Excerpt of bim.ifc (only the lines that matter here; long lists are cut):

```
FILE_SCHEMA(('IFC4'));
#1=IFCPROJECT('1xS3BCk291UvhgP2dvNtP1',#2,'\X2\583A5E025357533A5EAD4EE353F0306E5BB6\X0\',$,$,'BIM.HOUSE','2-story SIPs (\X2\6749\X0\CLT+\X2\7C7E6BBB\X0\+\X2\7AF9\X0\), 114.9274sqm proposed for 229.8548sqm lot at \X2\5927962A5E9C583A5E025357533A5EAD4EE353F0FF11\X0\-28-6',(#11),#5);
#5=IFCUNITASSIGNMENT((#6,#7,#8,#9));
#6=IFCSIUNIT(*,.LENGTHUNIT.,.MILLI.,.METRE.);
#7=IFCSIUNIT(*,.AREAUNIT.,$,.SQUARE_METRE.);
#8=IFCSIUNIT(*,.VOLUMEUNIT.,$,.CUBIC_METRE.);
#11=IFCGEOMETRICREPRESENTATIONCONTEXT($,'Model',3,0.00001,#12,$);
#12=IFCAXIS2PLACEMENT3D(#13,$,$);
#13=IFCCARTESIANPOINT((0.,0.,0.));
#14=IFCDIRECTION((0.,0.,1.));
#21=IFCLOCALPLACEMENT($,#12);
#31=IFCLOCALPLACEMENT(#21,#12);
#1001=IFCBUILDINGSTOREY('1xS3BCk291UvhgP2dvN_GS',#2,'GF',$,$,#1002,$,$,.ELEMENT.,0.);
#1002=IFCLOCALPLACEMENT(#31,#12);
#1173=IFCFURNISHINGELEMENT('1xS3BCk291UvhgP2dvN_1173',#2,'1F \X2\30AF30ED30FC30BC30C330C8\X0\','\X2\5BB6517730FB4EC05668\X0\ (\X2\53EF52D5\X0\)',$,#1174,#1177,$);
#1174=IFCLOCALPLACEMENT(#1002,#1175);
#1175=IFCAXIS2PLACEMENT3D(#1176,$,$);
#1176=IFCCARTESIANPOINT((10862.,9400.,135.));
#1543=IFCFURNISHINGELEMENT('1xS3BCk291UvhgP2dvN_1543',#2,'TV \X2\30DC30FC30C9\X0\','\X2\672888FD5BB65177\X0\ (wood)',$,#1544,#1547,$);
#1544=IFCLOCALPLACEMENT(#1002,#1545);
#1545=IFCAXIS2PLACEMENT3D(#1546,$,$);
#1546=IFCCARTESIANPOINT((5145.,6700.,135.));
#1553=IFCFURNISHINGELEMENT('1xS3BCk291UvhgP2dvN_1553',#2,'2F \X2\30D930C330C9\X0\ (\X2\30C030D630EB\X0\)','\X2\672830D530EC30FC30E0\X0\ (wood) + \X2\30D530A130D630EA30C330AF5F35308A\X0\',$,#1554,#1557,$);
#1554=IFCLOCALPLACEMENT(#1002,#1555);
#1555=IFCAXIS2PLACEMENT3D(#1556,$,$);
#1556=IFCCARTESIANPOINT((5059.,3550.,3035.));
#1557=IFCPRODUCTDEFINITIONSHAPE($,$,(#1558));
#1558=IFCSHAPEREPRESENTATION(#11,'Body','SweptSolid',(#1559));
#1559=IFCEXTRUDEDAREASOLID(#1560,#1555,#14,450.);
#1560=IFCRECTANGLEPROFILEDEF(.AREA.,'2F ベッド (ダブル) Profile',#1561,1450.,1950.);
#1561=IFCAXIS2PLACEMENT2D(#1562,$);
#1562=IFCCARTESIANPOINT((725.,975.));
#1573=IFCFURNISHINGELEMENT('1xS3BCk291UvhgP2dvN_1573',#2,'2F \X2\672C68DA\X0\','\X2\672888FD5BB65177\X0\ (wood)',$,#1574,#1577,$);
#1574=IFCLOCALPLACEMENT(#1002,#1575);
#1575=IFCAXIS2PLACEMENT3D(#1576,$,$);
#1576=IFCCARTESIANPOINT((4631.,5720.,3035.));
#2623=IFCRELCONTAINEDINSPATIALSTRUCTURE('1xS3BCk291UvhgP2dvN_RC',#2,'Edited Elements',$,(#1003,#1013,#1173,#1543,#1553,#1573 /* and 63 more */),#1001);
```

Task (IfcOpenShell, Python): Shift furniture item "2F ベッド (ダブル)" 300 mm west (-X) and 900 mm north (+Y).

```python
import ifcopenshell
import ifcopenshell.api.geometry
import ifcopenshell.util.placement

model = ifcopenshell.open("bim.ifc")

item = model.by_guid("1xS3BCk291UvhgP2dvN_1553")
matrix = ifcopenshell.util.placement.get_local_placement(item.ObjectPlacement)
matrix[0, 3] -= 300.0
matrix[1, 3] += 900.0
ifcopenshell.api.geometry.edit_object_placement(model, product=item, matrix=matrix, is_si=False)

print(ifcopenshell.util.placement.get_local_placement(item.ObjectPlacement).round(3) + 0.0)

model.write("bim_updated.ifc")
```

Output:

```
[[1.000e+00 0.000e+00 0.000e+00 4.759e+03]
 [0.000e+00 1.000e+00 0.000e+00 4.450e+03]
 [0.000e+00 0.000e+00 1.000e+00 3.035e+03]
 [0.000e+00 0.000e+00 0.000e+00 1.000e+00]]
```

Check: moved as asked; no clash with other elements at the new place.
